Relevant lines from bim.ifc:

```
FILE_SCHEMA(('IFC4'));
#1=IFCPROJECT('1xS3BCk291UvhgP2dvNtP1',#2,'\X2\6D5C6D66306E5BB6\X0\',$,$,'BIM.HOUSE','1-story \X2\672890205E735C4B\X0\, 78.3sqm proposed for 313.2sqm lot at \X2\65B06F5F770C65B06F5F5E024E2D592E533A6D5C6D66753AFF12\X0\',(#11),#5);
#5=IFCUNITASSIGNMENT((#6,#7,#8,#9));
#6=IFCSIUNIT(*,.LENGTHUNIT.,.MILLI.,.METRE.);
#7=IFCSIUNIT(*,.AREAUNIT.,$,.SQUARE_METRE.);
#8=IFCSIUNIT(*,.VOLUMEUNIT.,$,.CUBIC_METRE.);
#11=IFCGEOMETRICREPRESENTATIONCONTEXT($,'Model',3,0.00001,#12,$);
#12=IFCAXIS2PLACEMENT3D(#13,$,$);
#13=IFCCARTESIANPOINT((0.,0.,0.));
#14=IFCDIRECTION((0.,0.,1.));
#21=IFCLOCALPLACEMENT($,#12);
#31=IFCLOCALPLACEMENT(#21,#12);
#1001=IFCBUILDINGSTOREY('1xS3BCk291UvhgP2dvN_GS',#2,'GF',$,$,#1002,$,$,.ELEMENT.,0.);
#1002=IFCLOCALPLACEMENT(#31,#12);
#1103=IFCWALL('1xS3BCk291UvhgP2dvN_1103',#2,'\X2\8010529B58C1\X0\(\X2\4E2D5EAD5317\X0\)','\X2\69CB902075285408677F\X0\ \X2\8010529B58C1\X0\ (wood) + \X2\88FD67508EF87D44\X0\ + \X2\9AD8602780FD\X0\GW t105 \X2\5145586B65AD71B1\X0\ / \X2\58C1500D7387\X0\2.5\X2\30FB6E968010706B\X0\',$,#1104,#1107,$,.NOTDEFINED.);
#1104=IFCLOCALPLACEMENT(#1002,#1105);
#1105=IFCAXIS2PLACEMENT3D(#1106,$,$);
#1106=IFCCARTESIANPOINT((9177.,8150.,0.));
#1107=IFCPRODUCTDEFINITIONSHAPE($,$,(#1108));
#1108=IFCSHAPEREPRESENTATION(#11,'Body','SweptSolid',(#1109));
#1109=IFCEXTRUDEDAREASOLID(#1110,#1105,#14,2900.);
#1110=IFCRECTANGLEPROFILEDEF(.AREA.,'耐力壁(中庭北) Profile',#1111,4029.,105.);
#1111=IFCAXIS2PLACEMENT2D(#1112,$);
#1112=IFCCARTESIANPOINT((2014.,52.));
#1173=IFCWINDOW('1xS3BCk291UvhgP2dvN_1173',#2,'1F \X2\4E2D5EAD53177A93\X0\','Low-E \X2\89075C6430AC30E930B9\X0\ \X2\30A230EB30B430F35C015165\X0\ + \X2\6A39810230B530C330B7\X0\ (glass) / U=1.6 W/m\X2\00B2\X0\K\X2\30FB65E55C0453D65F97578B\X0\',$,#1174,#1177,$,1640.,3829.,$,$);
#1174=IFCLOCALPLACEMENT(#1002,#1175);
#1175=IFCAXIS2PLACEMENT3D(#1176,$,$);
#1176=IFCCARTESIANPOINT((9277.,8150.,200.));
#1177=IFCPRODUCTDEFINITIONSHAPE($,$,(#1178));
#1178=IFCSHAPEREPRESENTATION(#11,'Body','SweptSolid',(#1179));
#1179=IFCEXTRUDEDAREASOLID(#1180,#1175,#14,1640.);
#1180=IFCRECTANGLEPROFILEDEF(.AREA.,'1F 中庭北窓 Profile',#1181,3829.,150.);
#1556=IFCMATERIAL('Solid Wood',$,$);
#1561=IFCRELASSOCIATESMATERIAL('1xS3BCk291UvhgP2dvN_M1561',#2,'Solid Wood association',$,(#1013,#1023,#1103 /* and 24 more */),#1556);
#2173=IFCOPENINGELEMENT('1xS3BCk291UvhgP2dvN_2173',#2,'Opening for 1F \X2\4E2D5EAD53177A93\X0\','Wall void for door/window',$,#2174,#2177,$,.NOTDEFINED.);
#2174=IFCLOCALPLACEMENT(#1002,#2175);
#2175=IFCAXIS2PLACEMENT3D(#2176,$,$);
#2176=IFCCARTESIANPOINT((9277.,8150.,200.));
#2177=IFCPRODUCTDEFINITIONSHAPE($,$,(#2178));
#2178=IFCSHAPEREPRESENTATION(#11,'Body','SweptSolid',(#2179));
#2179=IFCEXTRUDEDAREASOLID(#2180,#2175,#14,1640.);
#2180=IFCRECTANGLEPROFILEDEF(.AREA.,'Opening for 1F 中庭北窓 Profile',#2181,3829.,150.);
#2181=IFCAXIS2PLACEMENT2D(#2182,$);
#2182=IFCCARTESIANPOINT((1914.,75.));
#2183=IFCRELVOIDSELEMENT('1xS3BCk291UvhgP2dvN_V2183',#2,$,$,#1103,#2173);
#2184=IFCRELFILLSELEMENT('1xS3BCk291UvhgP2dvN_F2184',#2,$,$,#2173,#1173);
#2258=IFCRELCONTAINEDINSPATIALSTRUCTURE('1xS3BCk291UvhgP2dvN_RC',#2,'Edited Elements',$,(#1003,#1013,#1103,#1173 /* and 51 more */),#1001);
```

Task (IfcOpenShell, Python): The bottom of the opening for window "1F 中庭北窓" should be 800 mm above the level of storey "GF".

```python
import numpy as np
import ifcopenshell
import ifcopenshell.api.geometry
import ifcopenshell.geom
import ifcopenshell.util.element
import ifcopenshell.util.placement
import ifcopenshell.util.shape
import ifcopenshell.util.unit

model = ifcopenshell.open("bim.ifc")
unit_scale = ifcopenshell.util.unit.calculate_unit_scale(model)

window = model.by_guid("1xS3BCk291UvhgP2dvN_1173")
opening = window.FillsVoids[0].RelatingOpeningElement
storey = ifcopenshell.util.element.get_container(window, ifc_class="IfcBuildingStorey")
level = ifcopenshell.util.placement.get_local_placement(storey.ObjectPlacement)[2, 3]

# The opening's origin need not be at the sill, so measure its lowest point.
shape = ifcopenshell.geom.create_shape(ifcopenshell.geom.settings(), opening)
bottom = ifcopenshell.util.shape.get_shape_bottom_elevation(shape, shape.geometry) / unit_scale
dz = level + 800.0 - bottom

shift = np.array([0.0, 0.0, dz])
# The window is not placed relative to its opening, so move both.
for product in (opening, window):
    matrix = ifcopenshell.util.placement.get_local_placement(product.ObjectPlacement)
    matrix[:3, 3] += shift
    ifcopenshell.api.geometry.edit_object_placement(model, product=product, matrix=matrix, is_si=False)

print(f"moved by {dz * unit_scale:+.3f} m")

model.write("bim_edited.ifc")
```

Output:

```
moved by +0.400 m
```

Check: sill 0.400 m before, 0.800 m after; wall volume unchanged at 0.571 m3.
